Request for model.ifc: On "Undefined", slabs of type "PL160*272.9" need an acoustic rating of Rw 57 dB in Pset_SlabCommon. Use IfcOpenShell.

First a look at what the model holds.

```python
import ifcopenshell
import ifcopenshell.util.element

model = ifcopenshell.open("model.ifc")
print(model.schema)
storey = next(s for s in model.by_type("IfcBuildingStorey") if s.Name == "Undefined")
slabs = [e for e in ifcopenshell.util.element.get_decomposition(storey) if e.is_a("IfcSlab")]
seen = {}
for e in slabs:
    element_type = ifcopenshell.util.element.get_type(e)
    key = (element_type.Name if element_type != e and element_type else None, ifcopenshell.util.element.get_pset(e, "Pset_SlabCommon", "AcousticRating"))
    seen[key] = seen.get(key, 0) + 1
for (name, value), count in sorted(seen.items(), key=str):
    print(count, "x", name, "|", value)
```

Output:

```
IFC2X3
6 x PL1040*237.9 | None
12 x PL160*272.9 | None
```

```python
import ifcopenshell
import ifcopenshell.api.pset
import ifcopenshell.util.element

model = ifcopenshell.open("model.ifc")

storey = next(s for s in model.by_type("IfcBuildingStorey") if s.Name == "Undefined")
slabs = [e for e in ifcopenshell.util.element.get_decomposition(storey) if e.is_a("IfcSlab")]

count = 0
for e in slabs:
    element_type = ifcopenshell.util.element.get_type(e)
    if element_type in (None, e) or element_type.Name != "PL160*272.9":
        continue
    # add_pset returns the element's existing set when there is one.
    pset = ifcopenshell.api.pset.add_pset(model, product=e, name="Pset_SlabCommon")
    ifcopenshell.api.pset.edit_pset(model, pset=pset, properties={"AcousticRating": "Rw 57 dB"})
    count += 1

print(count, "slabs updated")

model.write("model_updated.ifc")
```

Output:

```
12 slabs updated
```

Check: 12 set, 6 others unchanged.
